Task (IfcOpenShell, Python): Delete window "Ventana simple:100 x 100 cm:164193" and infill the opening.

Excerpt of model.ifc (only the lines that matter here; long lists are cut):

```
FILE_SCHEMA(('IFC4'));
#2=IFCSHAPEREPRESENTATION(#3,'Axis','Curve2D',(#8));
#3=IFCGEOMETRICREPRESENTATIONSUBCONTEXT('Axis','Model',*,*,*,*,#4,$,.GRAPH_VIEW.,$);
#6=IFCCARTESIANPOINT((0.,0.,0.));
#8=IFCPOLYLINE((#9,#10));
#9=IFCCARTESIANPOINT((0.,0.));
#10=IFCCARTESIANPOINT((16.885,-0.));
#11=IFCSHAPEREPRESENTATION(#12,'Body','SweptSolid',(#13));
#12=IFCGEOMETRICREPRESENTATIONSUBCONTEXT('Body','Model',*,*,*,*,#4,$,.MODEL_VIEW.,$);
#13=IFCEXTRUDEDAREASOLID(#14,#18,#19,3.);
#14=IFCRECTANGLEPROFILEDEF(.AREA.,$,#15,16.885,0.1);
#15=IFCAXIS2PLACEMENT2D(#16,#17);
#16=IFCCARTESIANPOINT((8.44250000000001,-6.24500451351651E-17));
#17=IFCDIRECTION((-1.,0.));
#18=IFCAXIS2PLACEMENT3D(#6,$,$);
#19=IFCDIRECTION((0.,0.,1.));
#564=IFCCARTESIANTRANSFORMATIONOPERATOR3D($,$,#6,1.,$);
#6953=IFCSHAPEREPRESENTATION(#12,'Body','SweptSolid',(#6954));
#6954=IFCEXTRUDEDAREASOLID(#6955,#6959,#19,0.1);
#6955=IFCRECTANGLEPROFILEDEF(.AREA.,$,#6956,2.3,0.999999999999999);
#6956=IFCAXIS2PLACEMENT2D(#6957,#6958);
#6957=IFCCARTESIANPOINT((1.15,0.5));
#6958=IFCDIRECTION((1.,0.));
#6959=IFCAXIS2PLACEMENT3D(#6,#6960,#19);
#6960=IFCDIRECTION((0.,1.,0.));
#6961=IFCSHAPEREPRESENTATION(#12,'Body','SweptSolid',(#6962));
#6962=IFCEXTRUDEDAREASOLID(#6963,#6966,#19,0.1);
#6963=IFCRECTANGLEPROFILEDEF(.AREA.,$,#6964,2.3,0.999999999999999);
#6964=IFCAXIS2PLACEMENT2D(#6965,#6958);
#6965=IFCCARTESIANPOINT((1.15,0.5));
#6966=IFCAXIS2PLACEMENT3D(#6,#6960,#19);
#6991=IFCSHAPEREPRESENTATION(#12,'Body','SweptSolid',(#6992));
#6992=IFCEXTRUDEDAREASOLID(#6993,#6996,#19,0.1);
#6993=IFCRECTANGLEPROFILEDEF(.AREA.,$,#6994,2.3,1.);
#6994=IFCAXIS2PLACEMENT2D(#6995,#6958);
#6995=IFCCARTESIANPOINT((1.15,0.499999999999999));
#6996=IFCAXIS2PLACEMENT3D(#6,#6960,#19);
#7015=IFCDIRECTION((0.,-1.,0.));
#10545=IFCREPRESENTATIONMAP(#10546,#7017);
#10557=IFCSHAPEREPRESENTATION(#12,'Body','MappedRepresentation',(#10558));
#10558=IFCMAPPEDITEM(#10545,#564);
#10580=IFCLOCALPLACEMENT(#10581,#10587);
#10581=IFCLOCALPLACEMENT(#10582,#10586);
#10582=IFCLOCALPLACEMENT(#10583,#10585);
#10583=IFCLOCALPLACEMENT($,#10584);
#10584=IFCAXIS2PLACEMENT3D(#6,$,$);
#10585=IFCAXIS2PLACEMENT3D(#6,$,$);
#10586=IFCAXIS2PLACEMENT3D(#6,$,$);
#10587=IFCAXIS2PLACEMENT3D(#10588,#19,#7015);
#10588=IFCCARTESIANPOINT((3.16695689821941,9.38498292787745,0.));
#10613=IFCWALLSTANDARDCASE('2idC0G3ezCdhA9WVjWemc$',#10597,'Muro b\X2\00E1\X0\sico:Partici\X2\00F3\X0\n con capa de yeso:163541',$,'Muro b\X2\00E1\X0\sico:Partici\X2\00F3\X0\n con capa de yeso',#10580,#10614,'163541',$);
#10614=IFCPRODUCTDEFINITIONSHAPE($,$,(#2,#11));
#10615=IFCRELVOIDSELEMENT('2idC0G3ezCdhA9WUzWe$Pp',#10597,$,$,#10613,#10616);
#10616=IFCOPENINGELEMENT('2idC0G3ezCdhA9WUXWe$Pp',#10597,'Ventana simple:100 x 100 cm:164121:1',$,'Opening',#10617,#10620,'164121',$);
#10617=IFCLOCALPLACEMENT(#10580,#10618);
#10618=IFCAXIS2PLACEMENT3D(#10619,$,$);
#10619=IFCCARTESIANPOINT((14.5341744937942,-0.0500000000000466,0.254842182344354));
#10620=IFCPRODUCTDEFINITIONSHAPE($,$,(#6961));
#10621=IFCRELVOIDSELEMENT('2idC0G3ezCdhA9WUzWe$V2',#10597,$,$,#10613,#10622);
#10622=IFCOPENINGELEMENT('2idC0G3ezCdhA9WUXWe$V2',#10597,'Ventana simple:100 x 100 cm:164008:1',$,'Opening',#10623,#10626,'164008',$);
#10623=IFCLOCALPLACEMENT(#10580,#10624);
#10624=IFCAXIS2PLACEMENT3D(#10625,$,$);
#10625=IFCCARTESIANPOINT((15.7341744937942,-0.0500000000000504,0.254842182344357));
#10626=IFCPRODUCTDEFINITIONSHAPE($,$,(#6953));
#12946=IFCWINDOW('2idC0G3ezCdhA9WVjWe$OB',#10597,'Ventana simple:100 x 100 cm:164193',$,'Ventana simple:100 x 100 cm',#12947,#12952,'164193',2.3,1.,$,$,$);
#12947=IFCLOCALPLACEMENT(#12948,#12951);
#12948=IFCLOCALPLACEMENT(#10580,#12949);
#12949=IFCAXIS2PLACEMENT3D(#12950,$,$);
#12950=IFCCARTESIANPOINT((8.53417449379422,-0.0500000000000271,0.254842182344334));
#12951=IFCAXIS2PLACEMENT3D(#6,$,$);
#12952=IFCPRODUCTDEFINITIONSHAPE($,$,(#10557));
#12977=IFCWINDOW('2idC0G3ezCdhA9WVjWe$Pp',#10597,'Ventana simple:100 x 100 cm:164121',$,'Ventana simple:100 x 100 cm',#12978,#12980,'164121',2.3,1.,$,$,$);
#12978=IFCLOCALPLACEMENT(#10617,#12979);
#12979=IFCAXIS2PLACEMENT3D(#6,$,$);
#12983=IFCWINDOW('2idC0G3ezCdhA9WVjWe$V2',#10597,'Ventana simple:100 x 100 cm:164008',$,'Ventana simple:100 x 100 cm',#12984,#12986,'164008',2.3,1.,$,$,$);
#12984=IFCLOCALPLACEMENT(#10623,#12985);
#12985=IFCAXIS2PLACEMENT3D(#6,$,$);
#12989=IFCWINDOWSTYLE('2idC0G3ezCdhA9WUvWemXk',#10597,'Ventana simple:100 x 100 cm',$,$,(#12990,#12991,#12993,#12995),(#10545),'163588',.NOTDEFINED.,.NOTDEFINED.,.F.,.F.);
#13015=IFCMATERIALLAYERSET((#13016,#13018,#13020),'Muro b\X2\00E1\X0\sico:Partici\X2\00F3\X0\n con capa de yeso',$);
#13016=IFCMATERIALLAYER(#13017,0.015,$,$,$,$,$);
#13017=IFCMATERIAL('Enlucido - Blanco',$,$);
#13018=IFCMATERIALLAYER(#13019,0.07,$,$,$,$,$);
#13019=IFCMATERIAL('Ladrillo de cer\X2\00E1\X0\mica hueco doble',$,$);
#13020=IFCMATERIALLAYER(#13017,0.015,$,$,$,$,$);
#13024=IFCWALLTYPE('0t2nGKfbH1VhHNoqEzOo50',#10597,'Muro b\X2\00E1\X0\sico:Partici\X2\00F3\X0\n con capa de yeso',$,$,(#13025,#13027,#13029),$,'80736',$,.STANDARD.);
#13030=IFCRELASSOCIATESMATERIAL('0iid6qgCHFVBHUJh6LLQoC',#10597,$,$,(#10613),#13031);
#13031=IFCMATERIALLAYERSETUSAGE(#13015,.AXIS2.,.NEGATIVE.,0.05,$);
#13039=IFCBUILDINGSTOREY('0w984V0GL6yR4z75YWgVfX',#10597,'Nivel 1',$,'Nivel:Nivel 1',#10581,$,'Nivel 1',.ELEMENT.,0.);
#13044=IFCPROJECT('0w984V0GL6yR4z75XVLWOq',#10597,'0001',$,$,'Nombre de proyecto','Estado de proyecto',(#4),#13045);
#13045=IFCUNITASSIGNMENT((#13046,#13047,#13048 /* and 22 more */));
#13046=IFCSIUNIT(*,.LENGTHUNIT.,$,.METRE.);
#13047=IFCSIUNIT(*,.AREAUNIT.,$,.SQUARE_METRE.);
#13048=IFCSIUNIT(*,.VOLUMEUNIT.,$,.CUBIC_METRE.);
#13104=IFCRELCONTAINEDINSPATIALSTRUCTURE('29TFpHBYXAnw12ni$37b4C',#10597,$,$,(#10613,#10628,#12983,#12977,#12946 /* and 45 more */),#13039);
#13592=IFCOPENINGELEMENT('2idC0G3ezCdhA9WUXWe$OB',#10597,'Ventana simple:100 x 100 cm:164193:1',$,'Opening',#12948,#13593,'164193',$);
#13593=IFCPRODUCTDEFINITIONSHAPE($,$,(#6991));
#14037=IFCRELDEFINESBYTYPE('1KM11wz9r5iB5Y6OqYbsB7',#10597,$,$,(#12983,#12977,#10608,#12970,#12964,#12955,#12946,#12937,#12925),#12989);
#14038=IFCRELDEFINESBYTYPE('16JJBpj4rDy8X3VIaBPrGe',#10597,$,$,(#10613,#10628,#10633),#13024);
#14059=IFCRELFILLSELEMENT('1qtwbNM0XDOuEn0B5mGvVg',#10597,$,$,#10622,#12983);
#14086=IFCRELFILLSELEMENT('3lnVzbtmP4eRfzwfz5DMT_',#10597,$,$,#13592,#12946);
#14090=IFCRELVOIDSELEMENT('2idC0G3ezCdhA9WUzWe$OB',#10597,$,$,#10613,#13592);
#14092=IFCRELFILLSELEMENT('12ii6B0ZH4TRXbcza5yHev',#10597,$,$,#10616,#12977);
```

```python
import ifcopenshell
import ifcopenshell.api.feature
import ifcopenshell.api.root
import ifcopenshell.geom
import ifcopenshell.util.shape

model = ifcopenshell.open("model.ifc")
settings = ifcopenshell.geom.settings()


def volume(element):
    """Net volume in cubic metres, openings subtracted."""
    shape = ifcopenshell.geom.create_shape(settings, element)
    return ifcopenshell.util.shape.get_volume(shape.geometry)


window = model.by_guid("2idC0G3ezCdhA9WVjWe$OB")
opening = window.FillsVoids[0].RelatingOpeningElement
wall = opening.VoidsElements[0].RelatingBuildingElement
before = volume(wall)

ifcopenshell.api.root.remove_product(model, product=window)
ifcopenshell.api.feature.remove_feature(model, feature=opening)

after = volume(wall)

print(f"wall volume {before:.3f} -> {after:.3f} m3")

model.write("model_v2.ifc")
```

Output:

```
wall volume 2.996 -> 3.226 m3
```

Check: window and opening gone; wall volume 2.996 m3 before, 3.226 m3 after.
